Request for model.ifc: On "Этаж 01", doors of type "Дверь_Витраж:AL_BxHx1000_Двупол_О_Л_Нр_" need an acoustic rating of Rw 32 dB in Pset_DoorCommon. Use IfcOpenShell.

First a look at what the model holds.

```python
import ifcopenshell
import ifcopenshell.util.element

model = ifcopenshell.open("model.ifc")
print(model.schema)
storey = next(s for s in model.by_type("IfcBuildingStorey") if s.Name == "Этаж 01")
doors = [e for e in ifcopenshell.util.element.get_decomposition(storey) if e.is_a("IfcDoor")]
seen = {}
for e in doors:
    element_type = ifcopenshell.util.element.get_type(e)
    key = (element_type.Name if element_type != e and element_type else None, ifcopenshell.util.element.get_pset(e, "Pset_DoorCommon", "AcousticRating"))
    seen[key] = seen.get(key, 0) + 1
for (name, value), count in sorted(seen.items(), key=str):
    print(count, "x", name, "|", value)
```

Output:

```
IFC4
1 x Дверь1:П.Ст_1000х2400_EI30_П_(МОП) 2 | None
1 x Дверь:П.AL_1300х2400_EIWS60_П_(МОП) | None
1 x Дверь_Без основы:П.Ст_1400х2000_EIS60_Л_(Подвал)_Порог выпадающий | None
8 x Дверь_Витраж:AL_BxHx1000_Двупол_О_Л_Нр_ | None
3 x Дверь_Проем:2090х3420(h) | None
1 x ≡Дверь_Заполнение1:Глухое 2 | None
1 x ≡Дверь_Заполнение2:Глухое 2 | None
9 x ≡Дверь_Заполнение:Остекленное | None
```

```python
import ifcopenshell
import ifcopenshell.api.pset
import ifcopenshell.util.element

model = ifcopenshell.open("model.ifc")

storey = next(s for s in model.by_type("IfcBuildingStorey") if s.Name == "Этаж 01")
doors = [e for e in ifcopenshell.util.element.get_decomposition(storey) if e.is_a("IfcDoor")]

count = 0
for e in doors:
    element_type = ifcopenshell.util.element.get_type(e)
    if element_type in (None, e) or element_type.Name != "Дверь_Витраж:AL_BxHx1000_Двупол_О_Л_Нр_":
        continue
    # add_pset returns the element's existing set when there is one.
    pset = ifcopenshell.api.pset.add_pset(model, product=e, name="Pset_DoorCommon")
    ifcopenshell.api.pset.edit_pset(model, pset=pset, properties={"AcousticRating": "Rw 32 dB"})
    count += 1

print(count, "doors updated")

model.write("model_v2.ifc")
```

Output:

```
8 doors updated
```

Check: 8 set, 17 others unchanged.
